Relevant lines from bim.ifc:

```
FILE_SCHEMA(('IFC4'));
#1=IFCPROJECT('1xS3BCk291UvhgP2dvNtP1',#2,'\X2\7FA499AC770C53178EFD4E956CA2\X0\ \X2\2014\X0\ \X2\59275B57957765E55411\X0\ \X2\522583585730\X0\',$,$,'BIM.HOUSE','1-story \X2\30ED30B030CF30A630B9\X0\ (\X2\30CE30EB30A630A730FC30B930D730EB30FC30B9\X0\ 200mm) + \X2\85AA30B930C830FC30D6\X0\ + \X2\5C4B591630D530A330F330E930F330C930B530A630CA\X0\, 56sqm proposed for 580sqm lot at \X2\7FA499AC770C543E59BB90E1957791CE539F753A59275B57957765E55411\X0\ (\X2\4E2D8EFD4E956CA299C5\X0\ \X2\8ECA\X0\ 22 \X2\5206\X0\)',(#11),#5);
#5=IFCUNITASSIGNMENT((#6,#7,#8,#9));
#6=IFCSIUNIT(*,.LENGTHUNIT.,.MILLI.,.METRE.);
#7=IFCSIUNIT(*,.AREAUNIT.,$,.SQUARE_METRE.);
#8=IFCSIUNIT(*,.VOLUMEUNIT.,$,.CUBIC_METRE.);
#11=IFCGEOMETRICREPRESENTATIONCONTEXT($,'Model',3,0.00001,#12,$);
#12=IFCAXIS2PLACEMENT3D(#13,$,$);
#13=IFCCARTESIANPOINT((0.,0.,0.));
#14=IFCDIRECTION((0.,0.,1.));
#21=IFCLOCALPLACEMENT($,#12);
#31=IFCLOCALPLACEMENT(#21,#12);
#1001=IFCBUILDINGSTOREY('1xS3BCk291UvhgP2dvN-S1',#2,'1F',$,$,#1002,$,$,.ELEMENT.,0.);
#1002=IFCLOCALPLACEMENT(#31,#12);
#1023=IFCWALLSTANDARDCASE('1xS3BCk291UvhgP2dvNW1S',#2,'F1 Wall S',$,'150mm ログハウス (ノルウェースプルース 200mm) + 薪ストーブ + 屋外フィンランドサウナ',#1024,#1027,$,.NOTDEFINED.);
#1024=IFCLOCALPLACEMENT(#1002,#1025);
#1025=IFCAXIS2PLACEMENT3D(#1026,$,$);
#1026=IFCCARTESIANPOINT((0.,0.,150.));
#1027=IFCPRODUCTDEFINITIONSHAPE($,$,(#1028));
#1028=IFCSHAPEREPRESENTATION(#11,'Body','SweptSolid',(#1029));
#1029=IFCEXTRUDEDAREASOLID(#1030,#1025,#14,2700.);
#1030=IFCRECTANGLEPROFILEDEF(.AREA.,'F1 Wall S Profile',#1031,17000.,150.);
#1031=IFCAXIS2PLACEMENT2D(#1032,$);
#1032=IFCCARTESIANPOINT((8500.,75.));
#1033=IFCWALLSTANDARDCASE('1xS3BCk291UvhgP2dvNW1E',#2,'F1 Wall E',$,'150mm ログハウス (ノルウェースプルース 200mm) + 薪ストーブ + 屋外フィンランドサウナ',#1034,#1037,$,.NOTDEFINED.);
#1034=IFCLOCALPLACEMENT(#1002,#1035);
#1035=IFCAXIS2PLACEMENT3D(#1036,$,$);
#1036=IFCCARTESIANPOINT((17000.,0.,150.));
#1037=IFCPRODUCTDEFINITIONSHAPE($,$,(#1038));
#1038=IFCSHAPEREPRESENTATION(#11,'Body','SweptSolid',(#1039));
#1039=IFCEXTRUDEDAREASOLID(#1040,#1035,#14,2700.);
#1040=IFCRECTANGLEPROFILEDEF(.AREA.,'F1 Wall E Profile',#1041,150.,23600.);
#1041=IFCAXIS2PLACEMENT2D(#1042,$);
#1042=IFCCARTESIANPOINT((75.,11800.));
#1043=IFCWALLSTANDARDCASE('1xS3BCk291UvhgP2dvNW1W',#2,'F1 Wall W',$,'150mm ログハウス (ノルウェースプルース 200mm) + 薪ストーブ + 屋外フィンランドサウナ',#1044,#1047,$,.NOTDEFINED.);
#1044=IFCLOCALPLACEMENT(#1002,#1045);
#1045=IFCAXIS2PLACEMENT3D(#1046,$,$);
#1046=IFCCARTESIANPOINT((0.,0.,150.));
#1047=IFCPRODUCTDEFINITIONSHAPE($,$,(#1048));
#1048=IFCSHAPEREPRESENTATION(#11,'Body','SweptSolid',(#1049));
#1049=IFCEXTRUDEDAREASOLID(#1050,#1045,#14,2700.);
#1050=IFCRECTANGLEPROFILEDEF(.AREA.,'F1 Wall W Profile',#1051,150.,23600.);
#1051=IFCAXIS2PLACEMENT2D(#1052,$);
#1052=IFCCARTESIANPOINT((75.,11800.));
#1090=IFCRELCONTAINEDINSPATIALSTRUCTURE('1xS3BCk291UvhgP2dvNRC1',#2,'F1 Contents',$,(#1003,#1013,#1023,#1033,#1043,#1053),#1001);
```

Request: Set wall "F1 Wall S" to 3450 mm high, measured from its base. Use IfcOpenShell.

```python
import ifcopenshell
import ifcopenshell.geom
import ifcopenshell.util.shape

model = ifcopenshell.open("bim.ifc")
settings = ifcopenshell.geom.settings()


def volume(element):
    """Net volume in cubic metres, openings subtracted."""
    shape = ifcopenshell.geom.create_shape(settings, element)
    return ifcopenshell.util.shape.get_volume(shape.geometry)


wall = model.by_guid("1xS3BCk291UvhgP2dvNW1S")
before = volume(wall)

body = next(r for r in wall.Representation.Representations if r.RepresentationIdentifier == "Body")
solid = body.Items[0]
old_height = solid.Depth
solid.Depth = 3450.0
after = volume(wall)

print(f"height {old_height:g} -> {solid.Depth:g}, volume {before:.3f} -> {after:.3f} m3")

model.write("bim_updated.ifc")
```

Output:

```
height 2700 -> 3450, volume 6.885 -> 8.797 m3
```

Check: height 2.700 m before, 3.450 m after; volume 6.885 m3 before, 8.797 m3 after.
